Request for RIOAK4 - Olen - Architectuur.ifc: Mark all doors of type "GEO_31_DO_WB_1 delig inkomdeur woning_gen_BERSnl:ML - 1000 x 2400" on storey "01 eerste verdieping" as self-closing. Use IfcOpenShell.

First a look at what the model holds.

```python
import ifcopenshell
import ifcopenshell.util.element

model = ifcopenshell.open("RIOAK4 - Olen - Architectuur.ifc")
print(model.schema)
storey = next(s for s in model.by_type("IfcBuildingStorey") if s.Name == "01 eerste verdieping")
doors = [e for e in ifcopenshell.util.element.get_decomposition(storey) if e.is_a("IfcDoor")]
seen = {}
for e in doors:
    element_type = ifcopenshell.util.element.get_type(e)
    key = (element_type.Name if element_type != e and element_type else None, ifcopenshell.util.element.get_pset(e, "Pset_DoorCommon", "SelfClosing"))
    seen[key] = seen.get(key, 0) + 1
for (name, value), count in sorted(seen.items(), key=str):
    print(count, "x", name, "|", value)
```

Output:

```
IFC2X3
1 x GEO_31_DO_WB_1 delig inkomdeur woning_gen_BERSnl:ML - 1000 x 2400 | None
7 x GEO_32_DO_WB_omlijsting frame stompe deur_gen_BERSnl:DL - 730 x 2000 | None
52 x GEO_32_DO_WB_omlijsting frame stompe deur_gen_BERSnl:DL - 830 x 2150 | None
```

```python
import ifcopenshell
import ifcopenshell.api.pset
import ifcopenshell.util.element

model = ifcopenshell.open("RIOAK4 - Olen - Architectuur.ifc")

storey = next(s for s in model.by_type("IfcBuildingStorey") if s.Name == "01 eerste verdieping")
doors = [e for e in ifcopenshell.util.element.get_decomposition(storey) if e.is_a("IfcDoor")]

count = 0
for e in doors:
    element_type = ifcopenshell.util.element.get_type(e)
    if element_type in (None, e) or element_type.Name != "GEO_31_DO_WB_1 delig inkomdeur woning_gen_BERSnl:ML - 1000 x 2400":
        continue
    # add_pset returns the element's existing set when there is one.
    pset = ifcopenshell.api.pset.add_pset(model, product=e, name="Pset_DoorCommon")
    ifcopenshell.api.pset.edit_pset(model, pset=pset, properties={"SelfClosing": True})
    count += 1

print(count, "doors updated")

model.write("RIOAK4 - Olen - Architectuur-out.ifc")
```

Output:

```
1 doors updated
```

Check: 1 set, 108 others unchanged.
